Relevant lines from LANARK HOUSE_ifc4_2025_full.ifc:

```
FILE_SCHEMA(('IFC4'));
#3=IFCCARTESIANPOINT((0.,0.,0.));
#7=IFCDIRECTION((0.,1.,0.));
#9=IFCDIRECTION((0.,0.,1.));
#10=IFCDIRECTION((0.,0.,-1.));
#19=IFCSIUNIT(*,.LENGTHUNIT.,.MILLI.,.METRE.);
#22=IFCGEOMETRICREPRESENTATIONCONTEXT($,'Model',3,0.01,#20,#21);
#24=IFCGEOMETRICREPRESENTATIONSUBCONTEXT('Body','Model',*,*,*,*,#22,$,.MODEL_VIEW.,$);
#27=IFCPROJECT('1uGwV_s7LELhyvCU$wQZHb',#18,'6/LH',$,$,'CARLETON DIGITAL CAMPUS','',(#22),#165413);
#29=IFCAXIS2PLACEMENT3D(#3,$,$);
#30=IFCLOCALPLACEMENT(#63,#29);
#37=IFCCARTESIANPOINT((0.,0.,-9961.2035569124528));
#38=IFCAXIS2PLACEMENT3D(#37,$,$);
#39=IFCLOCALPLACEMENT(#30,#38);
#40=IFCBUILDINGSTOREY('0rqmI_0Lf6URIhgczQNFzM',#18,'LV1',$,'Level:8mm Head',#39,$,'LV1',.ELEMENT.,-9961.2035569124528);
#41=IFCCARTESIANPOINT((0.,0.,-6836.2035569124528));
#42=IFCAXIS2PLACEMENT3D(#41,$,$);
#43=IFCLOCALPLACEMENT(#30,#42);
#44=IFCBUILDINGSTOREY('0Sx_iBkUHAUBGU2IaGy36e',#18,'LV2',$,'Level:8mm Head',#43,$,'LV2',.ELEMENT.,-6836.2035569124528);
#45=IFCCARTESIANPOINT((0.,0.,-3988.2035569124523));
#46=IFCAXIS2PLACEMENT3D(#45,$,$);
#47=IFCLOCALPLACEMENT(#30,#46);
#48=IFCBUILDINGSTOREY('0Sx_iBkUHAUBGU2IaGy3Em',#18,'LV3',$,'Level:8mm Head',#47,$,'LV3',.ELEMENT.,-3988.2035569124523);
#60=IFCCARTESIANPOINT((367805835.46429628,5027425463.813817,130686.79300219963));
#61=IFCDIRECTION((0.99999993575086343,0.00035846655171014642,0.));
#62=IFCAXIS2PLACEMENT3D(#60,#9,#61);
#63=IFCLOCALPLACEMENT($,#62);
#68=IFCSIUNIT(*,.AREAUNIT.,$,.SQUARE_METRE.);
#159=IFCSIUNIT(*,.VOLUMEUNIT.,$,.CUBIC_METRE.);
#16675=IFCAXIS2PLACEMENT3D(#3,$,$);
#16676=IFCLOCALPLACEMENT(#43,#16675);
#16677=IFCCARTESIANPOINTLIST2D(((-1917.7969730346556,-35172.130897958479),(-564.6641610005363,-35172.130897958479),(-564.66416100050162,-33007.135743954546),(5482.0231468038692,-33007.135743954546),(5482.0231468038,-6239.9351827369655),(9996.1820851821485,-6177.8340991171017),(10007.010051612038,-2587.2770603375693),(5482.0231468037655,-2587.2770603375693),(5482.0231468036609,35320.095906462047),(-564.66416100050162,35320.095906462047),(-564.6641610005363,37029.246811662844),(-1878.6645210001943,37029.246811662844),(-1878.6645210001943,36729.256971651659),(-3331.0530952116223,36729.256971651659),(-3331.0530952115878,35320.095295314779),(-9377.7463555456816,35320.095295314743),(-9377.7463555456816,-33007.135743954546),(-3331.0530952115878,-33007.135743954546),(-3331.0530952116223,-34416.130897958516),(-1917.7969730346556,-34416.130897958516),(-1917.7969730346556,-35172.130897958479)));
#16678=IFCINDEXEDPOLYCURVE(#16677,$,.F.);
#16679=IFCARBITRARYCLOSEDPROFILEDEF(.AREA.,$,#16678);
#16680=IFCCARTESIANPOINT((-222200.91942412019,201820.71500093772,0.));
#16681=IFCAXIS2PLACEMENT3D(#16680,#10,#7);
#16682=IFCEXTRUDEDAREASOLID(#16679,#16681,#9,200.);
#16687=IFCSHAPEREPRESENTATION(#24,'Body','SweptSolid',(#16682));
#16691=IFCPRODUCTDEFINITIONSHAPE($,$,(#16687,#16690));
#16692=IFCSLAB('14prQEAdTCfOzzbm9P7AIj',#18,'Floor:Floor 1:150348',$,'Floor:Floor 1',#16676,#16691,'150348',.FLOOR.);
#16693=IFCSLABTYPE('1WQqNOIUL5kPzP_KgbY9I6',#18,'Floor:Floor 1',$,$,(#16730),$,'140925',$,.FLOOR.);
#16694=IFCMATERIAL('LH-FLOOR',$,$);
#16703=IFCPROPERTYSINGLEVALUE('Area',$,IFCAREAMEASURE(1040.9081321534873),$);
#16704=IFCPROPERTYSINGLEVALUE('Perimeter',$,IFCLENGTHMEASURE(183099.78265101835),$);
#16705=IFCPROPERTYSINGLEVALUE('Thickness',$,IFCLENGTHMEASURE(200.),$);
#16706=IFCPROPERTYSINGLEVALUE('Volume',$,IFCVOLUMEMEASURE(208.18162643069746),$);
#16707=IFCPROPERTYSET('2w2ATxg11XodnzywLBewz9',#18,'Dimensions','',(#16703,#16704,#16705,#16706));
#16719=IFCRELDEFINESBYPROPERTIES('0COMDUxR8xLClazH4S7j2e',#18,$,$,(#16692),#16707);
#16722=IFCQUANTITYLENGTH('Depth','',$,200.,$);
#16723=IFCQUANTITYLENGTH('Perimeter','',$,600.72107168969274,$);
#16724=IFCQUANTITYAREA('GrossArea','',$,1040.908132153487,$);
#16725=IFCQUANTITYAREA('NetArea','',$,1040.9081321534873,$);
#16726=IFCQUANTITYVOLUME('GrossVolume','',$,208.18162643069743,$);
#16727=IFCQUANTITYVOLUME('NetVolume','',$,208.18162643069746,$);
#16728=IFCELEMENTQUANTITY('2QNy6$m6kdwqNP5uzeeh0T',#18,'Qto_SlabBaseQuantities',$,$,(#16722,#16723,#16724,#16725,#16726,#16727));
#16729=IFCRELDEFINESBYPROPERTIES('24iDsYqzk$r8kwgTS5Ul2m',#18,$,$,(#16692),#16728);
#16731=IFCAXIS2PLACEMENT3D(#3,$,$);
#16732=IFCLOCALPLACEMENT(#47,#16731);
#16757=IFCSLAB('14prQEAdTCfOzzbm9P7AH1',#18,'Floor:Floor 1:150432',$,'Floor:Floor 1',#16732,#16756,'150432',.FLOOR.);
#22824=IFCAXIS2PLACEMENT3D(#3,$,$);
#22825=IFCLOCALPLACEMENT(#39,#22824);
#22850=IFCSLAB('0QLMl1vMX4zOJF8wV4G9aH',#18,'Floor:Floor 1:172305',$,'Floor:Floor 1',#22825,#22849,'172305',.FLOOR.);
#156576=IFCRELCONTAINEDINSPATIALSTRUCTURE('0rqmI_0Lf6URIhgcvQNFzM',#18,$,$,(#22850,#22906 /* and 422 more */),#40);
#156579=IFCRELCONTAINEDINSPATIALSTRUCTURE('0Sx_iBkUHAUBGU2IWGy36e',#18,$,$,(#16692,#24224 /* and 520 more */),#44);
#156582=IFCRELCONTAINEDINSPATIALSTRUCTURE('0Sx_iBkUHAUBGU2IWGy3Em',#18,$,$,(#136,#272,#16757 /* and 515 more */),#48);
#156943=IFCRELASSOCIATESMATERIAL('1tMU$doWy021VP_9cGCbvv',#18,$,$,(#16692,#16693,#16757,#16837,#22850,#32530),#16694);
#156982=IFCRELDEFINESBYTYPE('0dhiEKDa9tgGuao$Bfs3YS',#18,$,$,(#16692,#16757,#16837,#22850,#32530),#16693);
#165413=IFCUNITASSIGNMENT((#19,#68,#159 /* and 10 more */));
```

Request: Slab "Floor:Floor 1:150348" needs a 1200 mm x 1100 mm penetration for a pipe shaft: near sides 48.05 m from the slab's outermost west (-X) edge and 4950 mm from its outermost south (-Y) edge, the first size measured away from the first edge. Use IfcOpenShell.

```python
import numpy as np
import ifcopenshell
import ifcopenshell.api.feature
import ifcopenshell.api.geometry
import ifcopenshell.api.pset
import ifcopenshell.api.root
import ifcopenshell.geom
import ifcopenshell.util.element
import ifcopenshell.util.placement
import ifcopenshell.util.representation
import ifcopenshell.util.shape
import ifcopenshell.util.unit

model = ifcopenshell.open("LANARK HOUSE_ifc4_2025_full.ifc")
unit_scale = ifcopenshell.util.unit.calculate_unit_scale(model)
area_scale = ifcopenshell.util.unit.calculate_unit_scale(model, "AREAUNIT")
volume_scale = ifcopenshell.util.unit.calculate_unit_scale(model, "VOLUMEUNIT")
settings = ifcopenshell.geom.settings()


def volume(element):
    """Net volume in cubic metres, openings subtracted."""
    shape = ifcopenshell.geom.create_shape(settings, element)
    return ifcopenshell.util.shape.get_volume(shape.geometry)


slab = model.by_id(16692)
before = volume(slab)

# Extent in the slab's own axes, in metres. The edges named are its -X and -Y sides.
slab_shape = ifcopenshell.geom.create_shape(settings, slab)
vertices = ifcopenshell.util.shape.get_vertices(slab_shape.geometry)
x_min, y_min, bottom = vertices.min(axis=0)
top = vertices[:, 2].max()

opening = ifcopenshell.api.root.create_entity(model, ifc_class="IfcOpeningElement", name="Pipe shaft opening", predefined_type="OPENING")
context = ifcopenshell.util.representation.get_context(model, "Model", "Body", "MODEL_VIEW")
width, depth = 1.2, 1.1
outline = [(0.0, 0.0), (width, 0.0), (width, depth), (0.0, depth), (0.0, 0.0)]
# Overshoot both faces by 50 mm so the cut is clean.
shape = ifcopenshell.api.geometry.add_slab_representation(
    model, context=context, depth=top - bottom + 0.1, polyline=outline
)
ifcopenshell.api.geometry.assign_representation(model, product=opening, representation=shape)

matrix = ifcopenshell.util.placement.get_local_placement(slab.ObjectPlacement)
matrix[:, 3] = matrix @ np.append(np.array([x_min + 48.05, y_min + 4.95, bottom - 0.05]) / unit_scale, 1.0)
ifcopenshell.api.geometry.edit_object_placement(model, product=opening, matrix=matrix, is_si=False)
ifcopenshell.api.feature.add_feature(model, feature=opening, element=slab)

after = volume(slab)

# Update the slab's stored quantities.
pset = model.by_id(ifcopenshell.util.element.get_pset(slab, "Dimensions", should_inherit=False)["id"])
ifcopenshell.api.pset.edit_pset(model, pset=pset, properties={
    "Area": model.create_entity("IfcAreaMeasure", after / (top - bottom) / area_scale),
    "Volume": model.create_entity("IfcVolumeMeasure", after / volume_scale),
})
qto = model.by_id(ifcopenshell.util.element.get_pset(slab, "Qto_SlabBaseQuantities", should_inherit=False)["id"])
ifcopenshell.api.pset.edit_qto(model, qto=qto, properties={
    "NetArea": after / (top - bottom) / area_scale,
    "NetVolume": after / volume_scale,
})

print(f"slab volume {before:.3f} -> {after:.3f} m3")

model.write("LANARK HOUSE_ifc4_2025_full_updated.ifc")
```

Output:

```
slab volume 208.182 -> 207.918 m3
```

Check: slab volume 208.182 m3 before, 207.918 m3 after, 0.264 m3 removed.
